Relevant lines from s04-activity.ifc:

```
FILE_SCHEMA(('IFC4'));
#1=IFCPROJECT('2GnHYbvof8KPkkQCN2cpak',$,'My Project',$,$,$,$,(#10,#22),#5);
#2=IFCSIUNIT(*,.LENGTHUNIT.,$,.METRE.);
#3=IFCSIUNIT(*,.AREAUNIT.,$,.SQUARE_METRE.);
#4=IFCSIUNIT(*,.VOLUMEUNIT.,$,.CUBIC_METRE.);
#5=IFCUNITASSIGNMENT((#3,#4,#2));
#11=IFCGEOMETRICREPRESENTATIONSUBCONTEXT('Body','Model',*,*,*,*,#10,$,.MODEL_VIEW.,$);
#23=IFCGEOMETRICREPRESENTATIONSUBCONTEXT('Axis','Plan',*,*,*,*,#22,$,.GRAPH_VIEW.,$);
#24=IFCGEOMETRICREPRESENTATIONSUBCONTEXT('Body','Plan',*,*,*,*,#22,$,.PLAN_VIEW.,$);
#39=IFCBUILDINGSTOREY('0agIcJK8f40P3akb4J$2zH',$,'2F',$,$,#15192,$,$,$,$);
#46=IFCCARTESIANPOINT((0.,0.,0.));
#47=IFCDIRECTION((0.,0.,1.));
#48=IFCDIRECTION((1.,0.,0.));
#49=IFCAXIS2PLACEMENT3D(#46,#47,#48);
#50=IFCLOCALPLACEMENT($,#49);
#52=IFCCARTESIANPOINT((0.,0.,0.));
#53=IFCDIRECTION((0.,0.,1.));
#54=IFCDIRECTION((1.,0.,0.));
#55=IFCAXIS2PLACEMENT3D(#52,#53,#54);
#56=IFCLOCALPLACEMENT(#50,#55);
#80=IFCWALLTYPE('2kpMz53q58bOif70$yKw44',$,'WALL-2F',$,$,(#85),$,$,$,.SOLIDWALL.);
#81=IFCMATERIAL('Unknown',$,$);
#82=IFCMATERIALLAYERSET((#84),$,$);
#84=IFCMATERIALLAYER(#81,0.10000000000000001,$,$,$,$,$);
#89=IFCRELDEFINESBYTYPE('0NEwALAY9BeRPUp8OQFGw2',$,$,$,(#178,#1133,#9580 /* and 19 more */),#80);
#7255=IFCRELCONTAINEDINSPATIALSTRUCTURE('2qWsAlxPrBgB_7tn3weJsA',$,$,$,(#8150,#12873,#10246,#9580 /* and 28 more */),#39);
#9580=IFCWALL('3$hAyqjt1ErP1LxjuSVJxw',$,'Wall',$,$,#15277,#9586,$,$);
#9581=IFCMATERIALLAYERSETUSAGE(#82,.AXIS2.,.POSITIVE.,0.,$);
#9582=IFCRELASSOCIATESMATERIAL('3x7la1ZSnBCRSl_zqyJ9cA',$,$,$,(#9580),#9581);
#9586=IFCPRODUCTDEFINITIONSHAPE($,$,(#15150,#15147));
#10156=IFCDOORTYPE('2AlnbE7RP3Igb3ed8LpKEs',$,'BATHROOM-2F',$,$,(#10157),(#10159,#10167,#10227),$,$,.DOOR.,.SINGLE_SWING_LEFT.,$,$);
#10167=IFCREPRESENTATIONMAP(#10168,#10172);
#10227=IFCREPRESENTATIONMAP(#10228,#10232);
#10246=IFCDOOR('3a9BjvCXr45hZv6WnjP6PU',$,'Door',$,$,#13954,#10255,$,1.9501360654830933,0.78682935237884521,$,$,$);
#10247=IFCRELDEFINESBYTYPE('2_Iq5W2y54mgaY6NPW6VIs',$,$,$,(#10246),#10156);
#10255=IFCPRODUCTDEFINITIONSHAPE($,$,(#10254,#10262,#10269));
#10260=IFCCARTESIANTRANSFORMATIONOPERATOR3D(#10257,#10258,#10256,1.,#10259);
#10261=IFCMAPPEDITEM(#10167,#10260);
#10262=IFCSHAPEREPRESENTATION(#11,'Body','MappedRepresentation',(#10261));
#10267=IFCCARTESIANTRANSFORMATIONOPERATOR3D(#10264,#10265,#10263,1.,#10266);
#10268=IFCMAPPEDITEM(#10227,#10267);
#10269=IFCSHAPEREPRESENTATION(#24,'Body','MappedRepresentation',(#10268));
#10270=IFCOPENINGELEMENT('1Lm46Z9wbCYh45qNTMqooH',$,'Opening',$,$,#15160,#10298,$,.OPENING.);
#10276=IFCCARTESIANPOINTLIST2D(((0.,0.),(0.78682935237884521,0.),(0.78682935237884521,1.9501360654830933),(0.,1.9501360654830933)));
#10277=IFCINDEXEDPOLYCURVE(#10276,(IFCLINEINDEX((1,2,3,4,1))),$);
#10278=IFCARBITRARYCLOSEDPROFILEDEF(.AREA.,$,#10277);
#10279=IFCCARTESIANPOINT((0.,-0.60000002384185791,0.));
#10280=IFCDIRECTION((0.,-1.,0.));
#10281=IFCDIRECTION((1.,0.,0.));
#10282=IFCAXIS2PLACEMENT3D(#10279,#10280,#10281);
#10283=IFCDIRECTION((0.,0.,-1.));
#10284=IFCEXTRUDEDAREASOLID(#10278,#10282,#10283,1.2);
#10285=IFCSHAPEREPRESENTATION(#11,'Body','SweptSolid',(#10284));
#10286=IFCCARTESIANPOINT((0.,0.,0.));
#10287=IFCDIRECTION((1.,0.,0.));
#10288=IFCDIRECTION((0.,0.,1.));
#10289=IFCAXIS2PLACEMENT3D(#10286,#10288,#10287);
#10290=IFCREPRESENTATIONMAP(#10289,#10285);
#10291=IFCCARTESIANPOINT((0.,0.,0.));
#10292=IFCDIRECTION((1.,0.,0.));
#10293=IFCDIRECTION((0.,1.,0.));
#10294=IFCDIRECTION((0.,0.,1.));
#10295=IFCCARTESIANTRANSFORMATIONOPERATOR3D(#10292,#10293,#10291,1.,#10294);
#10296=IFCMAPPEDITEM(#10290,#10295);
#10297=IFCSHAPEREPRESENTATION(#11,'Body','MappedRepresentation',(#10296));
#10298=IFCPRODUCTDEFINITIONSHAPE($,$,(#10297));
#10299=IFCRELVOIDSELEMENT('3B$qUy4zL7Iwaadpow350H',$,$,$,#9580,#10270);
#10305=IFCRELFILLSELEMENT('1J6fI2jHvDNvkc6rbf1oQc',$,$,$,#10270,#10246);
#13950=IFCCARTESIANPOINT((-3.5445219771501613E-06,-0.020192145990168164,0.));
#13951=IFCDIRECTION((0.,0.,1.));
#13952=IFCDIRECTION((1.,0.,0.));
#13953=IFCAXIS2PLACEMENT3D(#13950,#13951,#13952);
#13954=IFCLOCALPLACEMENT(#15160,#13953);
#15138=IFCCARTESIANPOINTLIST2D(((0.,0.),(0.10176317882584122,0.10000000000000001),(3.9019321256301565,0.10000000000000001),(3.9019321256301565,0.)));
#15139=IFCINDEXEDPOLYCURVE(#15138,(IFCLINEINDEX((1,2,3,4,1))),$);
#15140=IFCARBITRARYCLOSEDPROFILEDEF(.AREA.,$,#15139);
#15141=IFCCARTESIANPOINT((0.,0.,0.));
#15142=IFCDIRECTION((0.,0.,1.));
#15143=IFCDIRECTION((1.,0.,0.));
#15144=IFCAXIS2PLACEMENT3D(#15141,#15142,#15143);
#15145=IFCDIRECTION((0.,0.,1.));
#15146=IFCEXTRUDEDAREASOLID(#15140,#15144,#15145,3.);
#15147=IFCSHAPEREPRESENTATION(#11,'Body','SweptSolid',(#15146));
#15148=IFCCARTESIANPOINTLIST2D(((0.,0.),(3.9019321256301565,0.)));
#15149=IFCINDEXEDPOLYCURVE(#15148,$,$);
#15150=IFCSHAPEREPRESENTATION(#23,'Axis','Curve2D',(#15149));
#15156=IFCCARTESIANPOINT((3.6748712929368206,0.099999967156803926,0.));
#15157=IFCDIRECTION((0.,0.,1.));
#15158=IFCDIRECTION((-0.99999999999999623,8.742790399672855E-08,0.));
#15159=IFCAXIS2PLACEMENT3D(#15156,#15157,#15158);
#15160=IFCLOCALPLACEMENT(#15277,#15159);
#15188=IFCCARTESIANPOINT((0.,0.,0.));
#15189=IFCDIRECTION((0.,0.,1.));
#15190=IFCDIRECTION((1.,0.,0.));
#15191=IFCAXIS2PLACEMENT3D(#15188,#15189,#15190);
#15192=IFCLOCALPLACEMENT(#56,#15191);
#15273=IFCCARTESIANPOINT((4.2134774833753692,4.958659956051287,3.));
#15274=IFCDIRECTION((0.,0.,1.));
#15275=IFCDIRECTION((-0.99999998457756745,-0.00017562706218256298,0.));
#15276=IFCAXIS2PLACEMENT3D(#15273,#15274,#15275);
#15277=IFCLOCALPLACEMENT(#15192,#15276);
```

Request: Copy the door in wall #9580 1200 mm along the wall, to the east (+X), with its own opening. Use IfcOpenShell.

```python
import ifcopenshell
import ifcopenshell.api.feature
import ifcopenshell.api.geometry
import ifcopenshell.api.root
import ifcopenshell.geom
import ifcopenshell.util.element
import ifcopenshell.util.placement
import ifcopenshell.util.shape

model = ifcopenshell.open("s04-activity.ifc")
settings = ifcopenshell.geom.settings()


def volume(element):
    """Net volume in cubic metres, openings subtracted."""
    shape = ifcopenshell.geom.create_shape(settings, element)
    return ifcopenshell.util.shape.get_volume(shape.geometry)


door = model.by_guid("3a9BjvCXr45hZv6WnjP6PU")
opening = door.FillsVoids[0].RelatingOpeningElement
wall = opening.VoidsElements[0].RelatingBuildingElement
before = volume(wall)
shift = ifcopenshell.util.placement.get_local_placement(wall.ObjectPlacement)[:3, 0] * -1.2

# copy_class copies the void relationship, type, container and properties, but no geometry.
new_opening = ifcopenshell.api.root.copy_class(model, product=opening)
new_opening.Representation = ifcopenshell.util.element.copy_deep(
    model, opening.Representation, exclude=["IfcGeometricRepresentationContext", "IfcRepresentationMap"]
)
new_door = ifcopenshell.api.root.copy_class(model, product=door)
new_door.Representation = ifcopenshell.util.element.copy_deep(
    model, door.Representation, exclude=["IfcGeometricRepresentationContext", "IfcRepresentationMap"]
)
ifcopenshell.api.feature.add_filling(model, opening=new_opening, element=new_door)

for old, new in ((opening, new_opening), (door, new_door)):
    matrix = ifcopenshell.util.placement.get_local_placement(old.ObjectPlacement)
    matrix[:3, 3] += shift
    ifcopenshell.api.geometry.edit_object_placement(model, product=new, matrix=matrix, is_si=False)

after = volume(wall)

print(f"wall volume {before:.3f} -> {after:.3f} m3")

model.write("s04-activity_v2.ifc")
```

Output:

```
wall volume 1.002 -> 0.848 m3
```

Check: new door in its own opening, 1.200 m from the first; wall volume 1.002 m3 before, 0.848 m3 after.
